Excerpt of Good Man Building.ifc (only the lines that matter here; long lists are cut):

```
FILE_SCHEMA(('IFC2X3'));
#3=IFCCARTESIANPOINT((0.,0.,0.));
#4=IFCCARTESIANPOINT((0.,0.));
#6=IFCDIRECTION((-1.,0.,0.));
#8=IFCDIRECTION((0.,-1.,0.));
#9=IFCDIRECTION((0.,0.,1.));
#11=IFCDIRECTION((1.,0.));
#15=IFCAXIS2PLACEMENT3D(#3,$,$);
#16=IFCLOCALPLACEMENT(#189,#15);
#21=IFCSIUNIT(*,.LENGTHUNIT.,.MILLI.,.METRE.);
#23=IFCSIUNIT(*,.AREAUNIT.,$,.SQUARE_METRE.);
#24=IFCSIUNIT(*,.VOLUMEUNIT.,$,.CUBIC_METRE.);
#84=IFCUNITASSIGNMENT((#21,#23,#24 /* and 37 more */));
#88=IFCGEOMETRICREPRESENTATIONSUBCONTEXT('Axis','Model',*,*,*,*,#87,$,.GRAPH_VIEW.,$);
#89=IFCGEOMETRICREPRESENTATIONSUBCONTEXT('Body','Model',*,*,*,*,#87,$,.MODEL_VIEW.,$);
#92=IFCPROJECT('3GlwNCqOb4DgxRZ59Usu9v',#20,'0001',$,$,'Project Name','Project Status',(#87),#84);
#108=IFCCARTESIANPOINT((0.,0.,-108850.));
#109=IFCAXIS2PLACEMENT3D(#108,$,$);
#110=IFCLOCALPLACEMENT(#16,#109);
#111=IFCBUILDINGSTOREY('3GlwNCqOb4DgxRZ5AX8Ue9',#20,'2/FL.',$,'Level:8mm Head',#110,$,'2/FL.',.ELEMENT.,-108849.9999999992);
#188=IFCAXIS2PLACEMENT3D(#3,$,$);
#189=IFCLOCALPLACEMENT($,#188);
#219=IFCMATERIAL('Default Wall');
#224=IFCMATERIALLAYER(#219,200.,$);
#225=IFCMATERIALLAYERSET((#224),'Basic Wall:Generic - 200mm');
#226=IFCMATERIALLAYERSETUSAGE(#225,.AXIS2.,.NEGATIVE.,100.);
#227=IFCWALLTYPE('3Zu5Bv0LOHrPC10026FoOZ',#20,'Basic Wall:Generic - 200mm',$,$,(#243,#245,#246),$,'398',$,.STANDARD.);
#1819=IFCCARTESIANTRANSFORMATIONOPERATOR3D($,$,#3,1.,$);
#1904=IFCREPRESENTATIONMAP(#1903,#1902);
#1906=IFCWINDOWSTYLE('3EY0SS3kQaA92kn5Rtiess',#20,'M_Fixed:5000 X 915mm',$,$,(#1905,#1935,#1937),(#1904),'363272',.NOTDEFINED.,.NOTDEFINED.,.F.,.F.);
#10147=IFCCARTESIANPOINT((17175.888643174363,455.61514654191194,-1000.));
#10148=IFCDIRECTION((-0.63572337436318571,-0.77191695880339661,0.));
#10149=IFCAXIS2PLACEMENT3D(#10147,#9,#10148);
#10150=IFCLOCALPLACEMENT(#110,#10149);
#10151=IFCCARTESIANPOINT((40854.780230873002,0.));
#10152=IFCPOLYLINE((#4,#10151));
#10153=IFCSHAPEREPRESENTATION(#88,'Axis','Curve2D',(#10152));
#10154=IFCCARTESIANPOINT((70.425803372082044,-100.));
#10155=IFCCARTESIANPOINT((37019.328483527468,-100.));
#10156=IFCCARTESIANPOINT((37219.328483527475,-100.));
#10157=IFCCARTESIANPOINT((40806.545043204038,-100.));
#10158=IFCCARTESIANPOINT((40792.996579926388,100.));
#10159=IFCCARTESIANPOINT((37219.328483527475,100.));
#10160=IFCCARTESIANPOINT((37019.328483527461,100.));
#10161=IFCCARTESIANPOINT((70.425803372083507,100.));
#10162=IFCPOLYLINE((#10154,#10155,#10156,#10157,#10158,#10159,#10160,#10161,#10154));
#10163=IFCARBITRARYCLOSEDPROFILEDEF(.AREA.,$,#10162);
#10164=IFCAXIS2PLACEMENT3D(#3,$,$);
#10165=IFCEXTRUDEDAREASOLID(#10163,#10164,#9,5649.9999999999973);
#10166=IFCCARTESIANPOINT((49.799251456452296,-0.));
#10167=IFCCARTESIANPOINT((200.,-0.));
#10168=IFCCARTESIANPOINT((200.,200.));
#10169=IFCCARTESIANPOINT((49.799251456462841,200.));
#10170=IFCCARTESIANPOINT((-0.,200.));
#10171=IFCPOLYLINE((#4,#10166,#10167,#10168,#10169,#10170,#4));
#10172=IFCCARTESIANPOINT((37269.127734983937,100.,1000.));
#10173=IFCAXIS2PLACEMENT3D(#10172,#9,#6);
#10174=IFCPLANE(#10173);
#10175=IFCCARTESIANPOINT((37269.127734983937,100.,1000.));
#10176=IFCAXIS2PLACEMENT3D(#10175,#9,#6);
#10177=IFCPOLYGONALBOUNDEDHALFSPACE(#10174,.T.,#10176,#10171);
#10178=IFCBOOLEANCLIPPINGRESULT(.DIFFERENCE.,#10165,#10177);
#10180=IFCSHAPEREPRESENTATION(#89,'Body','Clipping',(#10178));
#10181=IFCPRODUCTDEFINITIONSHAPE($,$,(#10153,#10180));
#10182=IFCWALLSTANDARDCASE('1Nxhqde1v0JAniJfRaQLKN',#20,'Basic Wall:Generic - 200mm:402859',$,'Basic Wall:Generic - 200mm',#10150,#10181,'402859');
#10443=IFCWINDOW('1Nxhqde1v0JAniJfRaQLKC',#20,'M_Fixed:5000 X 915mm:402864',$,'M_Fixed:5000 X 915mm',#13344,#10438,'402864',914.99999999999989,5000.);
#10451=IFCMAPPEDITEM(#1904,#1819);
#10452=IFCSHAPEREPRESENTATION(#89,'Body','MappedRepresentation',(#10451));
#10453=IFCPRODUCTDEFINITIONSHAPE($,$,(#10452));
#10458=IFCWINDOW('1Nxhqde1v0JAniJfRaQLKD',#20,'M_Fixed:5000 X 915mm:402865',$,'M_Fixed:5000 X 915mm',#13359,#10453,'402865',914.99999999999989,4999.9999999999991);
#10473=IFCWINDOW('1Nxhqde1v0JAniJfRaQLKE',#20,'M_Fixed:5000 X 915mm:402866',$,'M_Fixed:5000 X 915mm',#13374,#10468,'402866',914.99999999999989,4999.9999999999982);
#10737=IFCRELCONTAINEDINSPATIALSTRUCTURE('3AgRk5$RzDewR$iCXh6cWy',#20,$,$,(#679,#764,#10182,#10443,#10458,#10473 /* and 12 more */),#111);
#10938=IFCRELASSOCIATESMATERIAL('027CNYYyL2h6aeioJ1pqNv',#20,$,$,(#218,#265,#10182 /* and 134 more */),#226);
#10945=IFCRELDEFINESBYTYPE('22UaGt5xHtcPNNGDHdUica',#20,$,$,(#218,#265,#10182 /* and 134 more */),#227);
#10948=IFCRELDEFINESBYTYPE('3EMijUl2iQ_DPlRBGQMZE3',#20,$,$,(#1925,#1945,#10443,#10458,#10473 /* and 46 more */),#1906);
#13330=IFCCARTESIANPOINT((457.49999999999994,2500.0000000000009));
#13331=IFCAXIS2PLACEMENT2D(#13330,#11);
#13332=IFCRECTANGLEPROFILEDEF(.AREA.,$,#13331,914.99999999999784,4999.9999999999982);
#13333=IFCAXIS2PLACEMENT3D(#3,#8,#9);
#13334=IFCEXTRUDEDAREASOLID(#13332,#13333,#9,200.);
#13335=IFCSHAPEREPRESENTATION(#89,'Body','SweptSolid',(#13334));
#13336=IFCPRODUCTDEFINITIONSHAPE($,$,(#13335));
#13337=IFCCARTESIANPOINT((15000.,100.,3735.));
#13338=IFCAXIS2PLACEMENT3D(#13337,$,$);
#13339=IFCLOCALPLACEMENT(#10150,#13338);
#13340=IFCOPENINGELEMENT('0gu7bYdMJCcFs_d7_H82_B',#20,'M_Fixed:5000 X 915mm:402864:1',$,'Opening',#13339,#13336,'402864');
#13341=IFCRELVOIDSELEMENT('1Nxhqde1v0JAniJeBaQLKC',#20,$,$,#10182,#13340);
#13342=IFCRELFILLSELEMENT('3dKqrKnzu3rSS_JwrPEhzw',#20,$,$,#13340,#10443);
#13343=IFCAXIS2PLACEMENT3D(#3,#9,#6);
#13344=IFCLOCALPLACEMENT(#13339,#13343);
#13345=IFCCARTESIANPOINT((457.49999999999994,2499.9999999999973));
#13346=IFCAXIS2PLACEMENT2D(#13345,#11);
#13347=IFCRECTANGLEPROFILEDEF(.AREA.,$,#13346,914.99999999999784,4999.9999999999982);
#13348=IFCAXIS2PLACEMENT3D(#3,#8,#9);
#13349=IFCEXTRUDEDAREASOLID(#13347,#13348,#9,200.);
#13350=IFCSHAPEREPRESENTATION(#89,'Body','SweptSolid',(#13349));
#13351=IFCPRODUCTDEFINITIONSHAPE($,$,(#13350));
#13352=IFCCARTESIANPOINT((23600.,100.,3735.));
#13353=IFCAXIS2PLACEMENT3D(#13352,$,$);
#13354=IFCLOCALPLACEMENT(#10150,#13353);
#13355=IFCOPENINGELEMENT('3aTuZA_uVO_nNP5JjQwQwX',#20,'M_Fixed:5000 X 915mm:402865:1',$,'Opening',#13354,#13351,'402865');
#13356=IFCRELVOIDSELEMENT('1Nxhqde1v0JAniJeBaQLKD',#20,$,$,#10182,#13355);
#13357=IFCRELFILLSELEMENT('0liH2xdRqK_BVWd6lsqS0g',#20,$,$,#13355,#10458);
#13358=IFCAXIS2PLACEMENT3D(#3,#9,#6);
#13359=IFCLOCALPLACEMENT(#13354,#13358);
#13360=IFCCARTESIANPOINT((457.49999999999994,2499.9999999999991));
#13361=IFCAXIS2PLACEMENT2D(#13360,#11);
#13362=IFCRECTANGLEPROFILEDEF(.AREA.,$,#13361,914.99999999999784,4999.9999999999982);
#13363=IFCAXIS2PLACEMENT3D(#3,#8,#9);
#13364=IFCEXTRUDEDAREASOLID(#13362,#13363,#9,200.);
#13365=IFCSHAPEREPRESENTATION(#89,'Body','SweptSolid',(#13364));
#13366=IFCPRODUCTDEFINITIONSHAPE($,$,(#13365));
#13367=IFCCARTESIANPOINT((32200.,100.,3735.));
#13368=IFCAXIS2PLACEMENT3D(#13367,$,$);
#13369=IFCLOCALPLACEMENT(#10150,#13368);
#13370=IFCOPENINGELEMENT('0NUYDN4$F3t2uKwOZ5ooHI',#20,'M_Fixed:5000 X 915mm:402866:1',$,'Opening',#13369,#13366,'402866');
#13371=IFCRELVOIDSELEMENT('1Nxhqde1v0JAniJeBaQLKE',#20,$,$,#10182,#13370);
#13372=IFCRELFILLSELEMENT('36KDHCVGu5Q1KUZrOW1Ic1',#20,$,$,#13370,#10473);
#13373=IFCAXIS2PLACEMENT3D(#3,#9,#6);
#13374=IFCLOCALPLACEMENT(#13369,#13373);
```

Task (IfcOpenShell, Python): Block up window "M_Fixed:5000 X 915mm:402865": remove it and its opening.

```python
import ifcopenshell
import ifcopenshell.api.feature
import ifcopenshell.api.root
import ifcopenshell.geom
import ifcopenshell.util.shape

model = ifcopenshell.open("Good Man Building.ifc")
settings = ifcopenshell.geom.settings()


def volume(element):
    """Net volume in cubic metres, openings subtracted."""
    shape = ifcopenshell.geom.create_shape(settings, element)
    return ifcopenshell.util.shape.get_volume(shape.geometry)


window = model.by_id(10458)
opening = window.FillsVoids[0].RelatingOpeningElement
wall = opening.VoidsElements[0].RelatingBuildingElement
before = volume(wall)

ifcopenshell.api.root.remove_product(model, product=window)
ifcopenshell.api.feature.remove_feature(model, feature=opening)

after = volume(wall)

print(f"wall volume {before:.3f} -> {after:.3f} m3")

model.write("Good Man Building_v2.ifc")
```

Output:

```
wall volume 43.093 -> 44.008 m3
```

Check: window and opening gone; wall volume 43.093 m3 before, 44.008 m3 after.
